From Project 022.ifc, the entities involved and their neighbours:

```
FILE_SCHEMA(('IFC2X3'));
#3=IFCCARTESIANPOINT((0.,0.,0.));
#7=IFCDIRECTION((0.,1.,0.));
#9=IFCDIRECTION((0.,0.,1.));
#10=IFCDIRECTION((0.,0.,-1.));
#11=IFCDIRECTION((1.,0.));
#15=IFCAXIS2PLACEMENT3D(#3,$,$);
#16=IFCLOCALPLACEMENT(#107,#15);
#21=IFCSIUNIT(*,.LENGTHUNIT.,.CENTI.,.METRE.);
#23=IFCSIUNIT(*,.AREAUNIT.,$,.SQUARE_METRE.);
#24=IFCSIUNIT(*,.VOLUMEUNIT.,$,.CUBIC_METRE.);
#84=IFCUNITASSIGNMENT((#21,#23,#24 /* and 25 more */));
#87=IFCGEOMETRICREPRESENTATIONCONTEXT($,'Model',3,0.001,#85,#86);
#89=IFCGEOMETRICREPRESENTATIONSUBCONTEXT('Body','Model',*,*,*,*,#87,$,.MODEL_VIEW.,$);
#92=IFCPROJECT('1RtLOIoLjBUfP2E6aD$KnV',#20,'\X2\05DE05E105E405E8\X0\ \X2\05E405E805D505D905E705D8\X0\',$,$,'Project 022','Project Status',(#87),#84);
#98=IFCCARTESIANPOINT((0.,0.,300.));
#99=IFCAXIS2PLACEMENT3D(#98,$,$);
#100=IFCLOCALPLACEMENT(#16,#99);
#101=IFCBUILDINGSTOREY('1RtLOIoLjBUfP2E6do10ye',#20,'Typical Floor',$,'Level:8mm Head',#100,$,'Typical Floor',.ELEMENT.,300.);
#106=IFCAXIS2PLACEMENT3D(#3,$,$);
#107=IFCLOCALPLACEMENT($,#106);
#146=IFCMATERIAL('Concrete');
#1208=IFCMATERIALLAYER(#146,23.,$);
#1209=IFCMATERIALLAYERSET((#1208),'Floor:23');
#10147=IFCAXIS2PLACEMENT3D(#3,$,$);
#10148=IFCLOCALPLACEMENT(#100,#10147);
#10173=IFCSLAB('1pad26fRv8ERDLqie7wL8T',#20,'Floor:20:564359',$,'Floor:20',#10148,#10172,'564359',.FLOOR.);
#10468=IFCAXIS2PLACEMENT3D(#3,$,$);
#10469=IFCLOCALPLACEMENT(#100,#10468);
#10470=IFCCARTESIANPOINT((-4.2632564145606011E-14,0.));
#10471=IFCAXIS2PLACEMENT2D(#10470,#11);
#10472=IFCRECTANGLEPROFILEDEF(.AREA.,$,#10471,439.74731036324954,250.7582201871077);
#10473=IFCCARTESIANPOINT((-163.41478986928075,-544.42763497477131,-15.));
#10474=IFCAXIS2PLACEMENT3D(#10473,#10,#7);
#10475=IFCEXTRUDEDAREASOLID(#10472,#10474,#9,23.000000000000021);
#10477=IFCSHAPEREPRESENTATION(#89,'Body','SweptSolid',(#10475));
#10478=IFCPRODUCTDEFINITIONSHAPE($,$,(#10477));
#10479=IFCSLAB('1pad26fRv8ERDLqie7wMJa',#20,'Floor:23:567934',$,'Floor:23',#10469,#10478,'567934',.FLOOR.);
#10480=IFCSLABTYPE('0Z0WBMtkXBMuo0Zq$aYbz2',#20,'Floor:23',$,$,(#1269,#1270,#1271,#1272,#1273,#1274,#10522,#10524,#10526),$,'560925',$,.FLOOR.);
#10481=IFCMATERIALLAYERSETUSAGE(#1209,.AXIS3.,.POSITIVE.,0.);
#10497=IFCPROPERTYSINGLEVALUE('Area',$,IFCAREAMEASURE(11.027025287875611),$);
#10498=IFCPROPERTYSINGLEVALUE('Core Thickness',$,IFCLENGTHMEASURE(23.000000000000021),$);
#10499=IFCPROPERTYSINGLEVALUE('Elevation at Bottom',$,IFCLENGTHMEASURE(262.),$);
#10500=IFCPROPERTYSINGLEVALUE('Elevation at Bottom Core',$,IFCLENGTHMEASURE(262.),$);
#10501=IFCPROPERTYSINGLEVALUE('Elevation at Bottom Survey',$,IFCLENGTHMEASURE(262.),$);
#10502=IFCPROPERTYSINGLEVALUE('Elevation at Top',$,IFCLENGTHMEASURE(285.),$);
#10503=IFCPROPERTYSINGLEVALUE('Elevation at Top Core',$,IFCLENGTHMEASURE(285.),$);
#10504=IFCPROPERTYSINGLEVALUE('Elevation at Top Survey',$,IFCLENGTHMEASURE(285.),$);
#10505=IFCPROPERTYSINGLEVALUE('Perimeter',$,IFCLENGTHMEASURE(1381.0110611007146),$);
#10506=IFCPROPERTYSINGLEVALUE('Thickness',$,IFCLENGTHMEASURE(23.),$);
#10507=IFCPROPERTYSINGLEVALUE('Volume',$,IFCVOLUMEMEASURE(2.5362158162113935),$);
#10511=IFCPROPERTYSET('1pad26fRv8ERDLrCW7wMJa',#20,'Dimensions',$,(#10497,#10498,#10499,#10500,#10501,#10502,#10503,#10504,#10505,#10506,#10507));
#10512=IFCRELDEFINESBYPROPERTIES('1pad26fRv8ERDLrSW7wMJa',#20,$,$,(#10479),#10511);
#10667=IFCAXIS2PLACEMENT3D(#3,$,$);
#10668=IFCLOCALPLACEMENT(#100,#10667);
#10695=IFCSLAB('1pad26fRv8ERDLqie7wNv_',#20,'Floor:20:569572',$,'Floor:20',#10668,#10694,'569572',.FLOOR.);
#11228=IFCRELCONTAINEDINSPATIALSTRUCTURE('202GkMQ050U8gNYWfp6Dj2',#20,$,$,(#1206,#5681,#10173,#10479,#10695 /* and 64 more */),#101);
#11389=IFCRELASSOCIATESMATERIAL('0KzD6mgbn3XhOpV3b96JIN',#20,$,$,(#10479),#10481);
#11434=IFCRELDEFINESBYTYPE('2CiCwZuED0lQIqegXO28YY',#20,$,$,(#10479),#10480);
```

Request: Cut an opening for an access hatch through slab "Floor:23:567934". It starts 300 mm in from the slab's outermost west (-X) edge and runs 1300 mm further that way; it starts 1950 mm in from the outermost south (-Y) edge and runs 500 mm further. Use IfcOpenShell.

```python
import numpy as np
import ifcopenshell
import ifcopenshell.api.feature
import ifcopenshell.api.geometry
import ifcopenshell.api.pset
import ifcopenshell.api.root
import ifcopenshell.geom
import ifcopenshell.util.element
import ifcopenshell.util.placement
import ifcopenshell.util.representation
import ifcopenshell.util.shape
import ifcopenshell.util.unit

model = ifcopenshell.open("Project 022.ifc")
unit_scale = ifcopenshell.util.unit.calculate_unit_scale(model)
area_scale = ifcopenshell.util.unit.calculate_unit_scale(model, "AREAUNIT")
volume_scale = ifcopenshell.util.unit.calculate_unit_scale(model, "VOLUMEUNIT")
settings = ifcopenshell.geom.settings()


def volume(element):
    """Net volume in cubic metres, openings subtracted."""
    shape = ifcopenshell.geom.create_shape(settings, element)
    return ifcopenshell.util.shape.get_volume(shape.geometry)


slab = model.by_guid("1pad26fRv8ERDLqie7wMJa")
before = volume(slab)

# Extent in the slab's own axes, in metres. The edges named are its -X and -Y sides.
slab_shape = ifcopenshell.geom.create_shape(settings, slab)
vertices = ifcopenshell.util.shape.get_vertices(slab_shape.geometry)
x_min, y_min, bottom = vertices.min(axis=0)
top = vertices[:, 2].max()

opening = ifcopenshell.api.root.create_entity(model, ifc_class="IfcOpeningElement", name="Access hatch opening")
context = ifcopenshell.util.representation.get_context(model, "Model", "Body", "MODEL_VIEW")
width, depth = 1.3, 0.5
outline = [(0.0, 0.0), (width, 0.0), (width, depth), (0.0, depth), (0.0, 0.0)]
# Overshoot both faces by 50 mm so the cut is clean.
shape = ifcopenshell.api.geometry.add_slab_representation(
    model, context=context, depth=top - bottom + 0.1, polyline=outline
)
ifcopenshell.api.geometry.assign_representation(model, product=opening, representation=shape)

matrix = ifcopenshell.util.placement.get_local_placement(slab.ObjectPlacement)
matrix[:, 3] = matrix @ np.append(np.array([x_min + 0.3, y_min + 1.95, bottom - 0.05]) / unit_scale, 1.0)
ifcopenshell.api.geometry.edit_object_placement(model, product=opening, matrix=matrix, is_si=False)
ifcopenshell.api.feature.add_feature(model, feature=opening, element=slab)

after = volume(slab)

# Update the slab's stored quantities.
pset = model.by_id(ifcopenshell.util.element.get_pset(slab, "Dimensions", should_inherit=False)["id"])
ifcopenshell.api.pset.edit_pset(model, pset=pset, properties={
    "Area": model.create_entity("IfcAreaMeasure", after / (top - bottom) / area_scale),
    "Volume": model.create_entity("IfcVolumeMeasure", after / volume_scale),
})

print(f"slab volume {before:.3f} -> {after:.3f} m3")

model.write("Project 022_updated.ifc")
```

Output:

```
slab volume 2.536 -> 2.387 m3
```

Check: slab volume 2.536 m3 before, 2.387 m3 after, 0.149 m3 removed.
